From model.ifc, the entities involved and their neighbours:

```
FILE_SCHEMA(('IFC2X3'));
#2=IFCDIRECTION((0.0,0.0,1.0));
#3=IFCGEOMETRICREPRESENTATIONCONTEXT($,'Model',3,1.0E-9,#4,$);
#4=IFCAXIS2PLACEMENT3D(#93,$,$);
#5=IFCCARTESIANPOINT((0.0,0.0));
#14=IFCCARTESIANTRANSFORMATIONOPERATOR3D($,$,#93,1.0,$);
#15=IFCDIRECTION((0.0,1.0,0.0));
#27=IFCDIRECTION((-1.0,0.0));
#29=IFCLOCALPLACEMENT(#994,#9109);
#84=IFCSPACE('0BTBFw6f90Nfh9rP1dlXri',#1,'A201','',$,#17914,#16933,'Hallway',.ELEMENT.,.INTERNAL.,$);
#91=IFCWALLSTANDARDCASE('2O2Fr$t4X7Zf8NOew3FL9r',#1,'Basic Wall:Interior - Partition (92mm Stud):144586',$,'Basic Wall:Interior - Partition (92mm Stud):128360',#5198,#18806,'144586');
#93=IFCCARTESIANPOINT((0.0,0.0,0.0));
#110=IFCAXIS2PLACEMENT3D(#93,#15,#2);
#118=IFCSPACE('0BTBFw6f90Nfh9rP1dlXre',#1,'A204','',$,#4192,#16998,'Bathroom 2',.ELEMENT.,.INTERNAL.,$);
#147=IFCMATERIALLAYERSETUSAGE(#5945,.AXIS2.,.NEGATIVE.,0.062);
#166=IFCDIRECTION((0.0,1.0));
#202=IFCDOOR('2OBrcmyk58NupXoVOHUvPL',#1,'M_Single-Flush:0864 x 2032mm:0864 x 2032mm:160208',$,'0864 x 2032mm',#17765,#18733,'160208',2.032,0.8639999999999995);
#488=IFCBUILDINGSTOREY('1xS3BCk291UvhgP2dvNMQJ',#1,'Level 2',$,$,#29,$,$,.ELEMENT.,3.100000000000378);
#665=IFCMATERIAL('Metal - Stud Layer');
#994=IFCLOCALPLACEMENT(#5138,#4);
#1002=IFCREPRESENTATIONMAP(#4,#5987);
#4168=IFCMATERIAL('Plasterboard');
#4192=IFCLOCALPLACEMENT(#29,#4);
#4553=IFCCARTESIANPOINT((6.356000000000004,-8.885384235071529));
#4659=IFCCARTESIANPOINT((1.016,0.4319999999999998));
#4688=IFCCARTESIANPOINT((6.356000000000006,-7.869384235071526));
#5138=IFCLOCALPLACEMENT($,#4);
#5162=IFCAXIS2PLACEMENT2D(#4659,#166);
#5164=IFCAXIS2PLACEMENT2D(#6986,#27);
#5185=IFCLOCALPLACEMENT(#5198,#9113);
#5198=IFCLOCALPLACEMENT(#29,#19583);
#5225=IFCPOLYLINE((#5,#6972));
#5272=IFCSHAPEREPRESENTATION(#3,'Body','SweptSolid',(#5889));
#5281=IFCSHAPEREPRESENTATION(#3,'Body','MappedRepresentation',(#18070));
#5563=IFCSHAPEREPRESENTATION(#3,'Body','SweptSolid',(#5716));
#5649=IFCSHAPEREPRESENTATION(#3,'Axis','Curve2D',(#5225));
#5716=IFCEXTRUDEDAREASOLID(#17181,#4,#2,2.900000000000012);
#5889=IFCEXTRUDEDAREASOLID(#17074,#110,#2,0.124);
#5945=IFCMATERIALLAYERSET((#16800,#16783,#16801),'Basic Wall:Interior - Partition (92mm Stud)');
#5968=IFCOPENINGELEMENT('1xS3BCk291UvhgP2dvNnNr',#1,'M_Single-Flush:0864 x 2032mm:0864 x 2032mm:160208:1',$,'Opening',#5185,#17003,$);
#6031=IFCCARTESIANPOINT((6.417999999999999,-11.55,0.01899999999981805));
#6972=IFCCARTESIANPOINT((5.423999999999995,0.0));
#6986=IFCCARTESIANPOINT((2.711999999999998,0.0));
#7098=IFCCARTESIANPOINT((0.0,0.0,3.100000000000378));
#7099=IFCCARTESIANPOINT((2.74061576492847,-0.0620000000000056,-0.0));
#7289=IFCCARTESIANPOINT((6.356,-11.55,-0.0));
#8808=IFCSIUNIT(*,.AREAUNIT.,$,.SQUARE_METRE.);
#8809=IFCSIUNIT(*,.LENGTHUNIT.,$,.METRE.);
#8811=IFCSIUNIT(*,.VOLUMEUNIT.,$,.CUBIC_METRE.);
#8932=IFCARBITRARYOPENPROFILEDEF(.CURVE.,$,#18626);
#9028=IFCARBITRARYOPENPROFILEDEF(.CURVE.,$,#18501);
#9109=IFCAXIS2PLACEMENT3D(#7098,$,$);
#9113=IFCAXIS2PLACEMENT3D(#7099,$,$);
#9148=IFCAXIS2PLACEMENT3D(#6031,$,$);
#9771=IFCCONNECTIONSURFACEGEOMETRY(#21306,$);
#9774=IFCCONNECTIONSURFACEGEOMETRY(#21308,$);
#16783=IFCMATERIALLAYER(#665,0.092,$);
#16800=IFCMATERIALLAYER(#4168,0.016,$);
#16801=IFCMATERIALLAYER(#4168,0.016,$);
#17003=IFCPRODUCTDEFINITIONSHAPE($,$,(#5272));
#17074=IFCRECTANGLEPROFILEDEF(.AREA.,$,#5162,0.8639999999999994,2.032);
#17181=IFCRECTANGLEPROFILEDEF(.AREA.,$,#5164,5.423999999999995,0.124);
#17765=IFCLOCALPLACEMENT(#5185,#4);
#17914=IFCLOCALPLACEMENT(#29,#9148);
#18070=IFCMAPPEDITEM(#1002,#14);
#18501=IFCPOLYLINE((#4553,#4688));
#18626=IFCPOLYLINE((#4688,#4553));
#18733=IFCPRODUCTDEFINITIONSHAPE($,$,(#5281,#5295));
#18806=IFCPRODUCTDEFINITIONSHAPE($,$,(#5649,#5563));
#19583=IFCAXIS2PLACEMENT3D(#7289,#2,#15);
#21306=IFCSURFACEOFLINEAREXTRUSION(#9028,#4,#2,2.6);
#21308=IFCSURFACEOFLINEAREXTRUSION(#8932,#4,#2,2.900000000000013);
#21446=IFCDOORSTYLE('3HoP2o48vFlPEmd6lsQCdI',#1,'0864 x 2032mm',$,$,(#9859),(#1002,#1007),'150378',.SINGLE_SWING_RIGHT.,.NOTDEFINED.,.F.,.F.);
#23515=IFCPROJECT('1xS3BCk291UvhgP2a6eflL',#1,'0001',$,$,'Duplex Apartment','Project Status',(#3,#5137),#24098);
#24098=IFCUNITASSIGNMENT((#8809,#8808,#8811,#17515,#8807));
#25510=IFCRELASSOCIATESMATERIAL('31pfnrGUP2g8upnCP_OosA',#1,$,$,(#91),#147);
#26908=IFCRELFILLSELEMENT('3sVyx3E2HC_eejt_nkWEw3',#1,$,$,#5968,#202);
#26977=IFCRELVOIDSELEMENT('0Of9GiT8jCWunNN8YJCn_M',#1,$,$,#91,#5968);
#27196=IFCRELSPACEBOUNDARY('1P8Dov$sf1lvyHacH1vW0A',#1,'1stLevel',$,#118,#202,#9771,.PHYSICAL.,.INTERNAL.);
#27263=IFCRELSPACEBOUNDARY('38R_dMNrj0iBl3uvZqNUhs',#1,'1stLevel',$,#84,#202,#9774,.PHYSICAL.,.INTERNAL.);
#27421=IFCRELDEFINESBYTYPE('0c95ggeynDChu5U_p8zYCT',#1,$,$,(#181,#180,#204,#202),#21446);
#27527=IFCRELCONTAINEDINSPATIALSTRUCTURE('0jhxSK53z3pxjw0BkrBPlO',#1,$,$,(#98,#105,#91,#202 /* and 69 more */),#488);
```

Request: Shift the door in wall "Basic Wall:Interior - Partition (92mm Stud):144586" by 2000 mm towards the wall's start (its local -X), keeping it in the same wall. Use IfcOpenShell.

```python
import numpy as np
import ifcopenshell
import ifcopenshell.api.geometry
import ifcopenshell.util.placement

model = ifcopenshell.open("model.ifc")

door = model.by_id(202)
opening = door.FillsVoids[0].RelatingOpeningElement
wall = opening.VoidsElements[0].RelatingBuildingElement

wall_matrix = ifcopenshell.util.placement.get_local_placement(wall.ObjectPlacement)
shift = wall_matrix[:3, 0] * -2.0
before = ifcopenshell.util.placement.get_local_placement(door.ObjectPlacement)[:3, 3].copy()

# The door is placed relative to its opening, so it follows when the opening moves.
matrix = ifcopenshell.util.placement.get_local_placement(opening.ObjectPlacement)
matrix[:3, 3] += shift
ifcopenshell.api.geometry.edit_object_placement(
    model, product=opening, matrix=matrix, is_si=False, should_transform_children=True
)

# Space boundary surfaces are stored in each space's coordinates; move them too.
for rel in door.ProvidesBoundaries:
    if not rel.ConnectionGeometry:
        continue
    surface = rel.ConnectionGeometry.SurfaceOnRelatingElement
    space_matrix = ifcopenshell.util.placement.get_local_placement(rel.RelatingSpace.ObjectPlacement)
    point = np.array(surface.Position.Location.Coordinates) + space_matrix[:3, :3].T @ shift
    surface.Position = model.createIfcAxis2Placement3D(
        model.createIfcCartesianPoint(point.tolist()), surface.Position.Axis, surface.Position.RefDirection
    )

after = ifcopenshell.util.placement.get_local_placement(door.ObjectPlacement)[:3, 3]
print("door moved by", (after - before).round(3) + 0.0)

model.write("model_v2.ifc")
```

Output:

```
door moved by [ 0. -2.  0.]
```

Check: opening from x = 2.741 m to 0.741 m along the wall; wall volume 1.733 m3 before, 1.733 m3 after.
